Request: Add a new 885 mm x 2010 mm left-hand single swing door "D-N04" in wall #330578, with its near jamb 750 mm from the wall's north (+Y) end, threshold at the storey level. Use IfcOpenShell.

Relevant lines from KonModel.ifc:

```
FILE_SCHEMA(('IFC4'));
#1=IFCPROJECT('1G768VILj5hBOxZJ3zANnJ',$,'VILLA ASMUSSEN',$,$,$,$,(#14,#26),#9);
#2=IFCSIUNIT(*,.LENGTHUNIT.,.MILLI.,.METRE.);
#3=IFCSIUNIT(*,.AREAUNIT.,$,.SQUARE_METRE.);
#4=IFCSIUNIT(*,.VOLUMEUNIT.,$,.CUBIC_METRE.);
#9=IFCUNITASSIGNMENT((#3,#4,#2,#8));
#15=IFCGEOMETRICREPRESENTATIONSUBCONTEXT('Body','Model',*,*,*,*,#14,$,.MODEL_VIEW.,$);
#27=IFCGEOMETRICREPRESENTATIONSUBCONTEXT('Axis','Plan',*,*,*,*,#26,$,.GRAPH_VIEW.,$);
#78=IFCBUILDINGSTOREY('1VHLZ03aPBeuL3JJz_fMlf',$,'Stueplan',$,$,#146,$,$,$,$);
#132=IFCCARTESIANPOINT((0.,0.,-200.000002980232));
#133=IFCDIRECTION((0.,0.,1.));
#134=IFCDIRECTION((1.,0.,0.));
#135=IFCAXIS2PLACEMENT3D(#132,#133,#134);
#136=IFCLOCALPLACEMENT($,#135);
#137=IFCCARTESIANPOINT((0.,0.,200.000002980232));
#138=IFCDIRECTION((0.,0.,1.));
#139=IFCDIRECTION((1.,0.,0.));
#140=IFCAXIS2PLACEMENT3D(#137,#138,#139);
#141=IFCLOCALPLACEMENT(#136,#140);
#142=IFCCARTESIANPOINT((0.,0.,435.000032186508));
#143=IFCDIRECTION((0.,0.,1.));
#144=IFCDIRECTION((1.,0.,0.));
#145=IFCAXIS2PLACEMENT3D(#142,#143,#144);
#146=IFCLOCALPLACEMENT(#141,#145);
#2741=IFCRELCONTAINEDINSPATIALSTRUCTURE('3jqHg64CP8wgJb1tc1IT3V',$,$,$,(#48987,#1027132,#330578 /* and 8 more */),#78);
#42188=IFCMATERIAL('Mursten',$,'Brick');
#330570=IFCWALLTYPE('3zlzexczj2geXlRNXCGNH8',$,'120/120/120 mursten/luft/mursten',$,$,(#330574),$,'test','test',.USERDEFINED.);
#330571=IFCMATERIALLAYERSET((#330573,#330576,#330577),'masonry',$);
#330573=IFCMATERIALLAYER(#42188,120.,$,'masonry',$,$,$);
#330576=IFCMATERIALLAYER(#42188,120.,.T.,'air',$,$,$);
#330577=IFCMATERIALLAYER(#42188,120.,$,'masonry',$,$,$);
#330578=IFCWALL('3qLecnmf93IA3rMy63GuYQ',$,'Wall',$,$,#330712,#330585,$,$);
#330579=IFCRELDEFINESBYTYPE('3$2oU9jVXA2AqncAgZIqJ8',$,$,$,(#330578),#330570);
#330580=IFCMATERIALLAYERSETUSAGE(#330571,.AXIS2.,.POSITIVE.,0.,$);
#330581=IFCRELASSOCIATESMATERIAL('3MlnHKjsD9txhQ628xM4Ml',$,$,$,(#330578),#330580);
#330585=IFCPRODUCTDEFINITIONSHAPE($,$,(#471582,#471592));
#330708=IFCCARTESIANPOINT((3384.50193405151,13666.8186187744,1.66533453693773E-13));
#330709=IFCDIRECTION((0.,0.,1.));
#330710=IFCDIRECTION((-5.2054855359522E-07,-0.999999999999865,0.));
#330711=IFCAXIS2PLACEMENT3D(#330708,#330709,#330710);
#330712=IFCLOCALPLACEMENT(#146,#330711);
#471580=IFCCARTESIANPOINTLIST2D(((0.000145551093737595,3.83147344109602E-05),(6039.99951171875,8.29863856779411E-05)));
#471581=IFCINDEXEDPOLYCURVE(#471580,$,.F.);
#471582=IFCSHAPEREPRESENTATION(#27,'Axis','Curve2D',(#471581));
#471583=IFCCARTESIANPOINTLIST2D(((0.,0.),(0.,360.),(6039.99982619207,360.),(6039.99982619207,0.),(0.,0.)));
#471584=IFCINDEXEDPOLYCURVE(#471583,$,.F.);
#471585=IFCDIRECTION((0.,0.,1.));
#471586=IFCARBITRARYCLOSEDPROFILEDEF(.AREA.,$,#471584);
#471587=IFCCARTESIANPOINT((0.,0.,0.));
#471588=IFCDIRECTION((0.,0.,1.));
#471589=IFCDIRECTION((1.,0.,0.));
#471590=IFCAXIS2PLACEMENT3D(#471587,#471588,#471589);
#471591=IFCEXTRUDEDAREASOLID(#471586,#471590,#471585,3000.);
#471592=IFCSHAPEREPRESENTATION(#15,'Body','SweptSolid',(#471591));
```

```python
import numpy as np
import ifcopenshell
import ifcopenshell.api.feature
import ifcopenshell.api.geometry
import ifcopenshell.api.root
import ifcopenshell.api.spatial
import ifcopenshell.geom
import ifcopenshell.util.element
import ifcopenshell.util.placement
import ifcopenshell.util.representation
import ifcopenshell.util.shape
import ifcopenshell.util.unit

model = ifcopenshell.open("KonModel.ifc")
unit_scale = ifcopenshell.util.unit.calculate_unit_scale(model)
settings = ifcopenshell.geom.settings()


def volume(element):
    """Net volume in cubic metres, openings subtracted."""
    shape = ifcopenshell.geom.create_shape(settings, element)
    return ifcopenshell.util.shape.get_volume(shape.geometry)


wall = model.by_id(330578)
storey = ifcopenshell.util.element.get_container(wall, ifc_class="IfcBuildingStorey")
context = ifcopenshell.util.representation.get_context(model, "Model", "Body", "MODEL_VIEW")
before = volume(wall)

width, height, from_end, sill = 0.885, 2.01, 0.75, 0.0  # metres

# The wall runs along its own X axis, and the end named is its -X end.
wall_shape = ifcopenshell.geom.create_shape(settings, wall)
x, y, z = ifcopenshell.util.shape.get_vertices(wall_shape.geometry).T
start = x.min() + from_end
face, thickness = float(y.min()), float(y.max() - y.min())
wall_matrix = ifcopenshell.util.placement.get_local_placement(wall.ObjectPlacement)
level = ifcopenshell.util.placement.get_local_placement(storey.ObjectPlacement)[2, 3]


def in_wall(x, y):
    """Placement at x, y metres in the wall's axes, at sill height."""
    matrix = wall_matrix.copy()
    matrix[:, 3] = wall_matrix @ np.array([x / unit_scale, y / unit_scale, 0.0, 1.0])
    matrix[2, 3] = level + sill / unit_scale
    return matrix


# Opening: a box that overshoots both wall faces by 50 mm.
opening = ifcopenshell.api.root.create_entity(model, ifc_class="IfcOpeningElement", predefined_type="OPENING")
box = ifcopenshell.api.geometry.add_wall_representation(
    model, context=context, length=width, height=height, thickness=thickness + 0.1
)
ifcopenshell.api.geometry.assign_representation(model, product=opening, representation=box)
ifcopenshell.api.geometry.edit_object_placement(model, product=opening, matrix=in_wall(start, face - 0.05), is_si=False)
ifcopenshell.api.feature.add_feature(model, feature=opening, element=wall)

door = ifcopenshell.api.root.create_entity(model, ifc_class="IfcDoor", name="D-N04", predefined_type="DOOR")
door.OverallWidth, door.OverallHeight = width / unit_scale, height / unit_scale
door.OperationType = "SINGLE_SWING_LEFT"
body = ifcopenshell.api.geometry.add_door_representation(
    model,
    context=context,
    overall_width=door.OverallWidth,
    overall_height=door.OverallHeight,
    operation_type="SINGLE_SWING_LEFT",
    lining_properties={"LiningDepth": thickness / unit_scale, "ThresholdDepth": thickness / unit_scale},
)
ifcopenshell.api.geometry.assign_representation(model, product=door, representation=body)
ifcopenshell.api.spatial.assign_container(model, products=[door], relating_structure=storey)
ifcopenshell.api.feature.add_filling(model, opening=opening, element=door)

# The lining spans the wall, so the door starts at the wall face.
ifcopenshell.api.geometry.edit_object_placement(model, product=door, matrix=in_wall(start, face), is_si=False)

after = volume(wall)

print(f"wall volume {before:.3f} -> {after:.3f} m3")

model.write("KonModel_rev.ifc")
```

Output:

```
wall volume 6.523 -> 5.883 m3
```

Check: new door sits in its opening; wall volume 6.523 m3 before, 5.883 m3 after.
